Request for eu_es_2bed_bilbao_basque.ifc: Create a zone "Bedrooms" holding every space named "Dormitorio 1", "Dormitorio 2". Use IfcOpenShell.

First a look at what the model holds.

```python
import ifcopenshell

model = ifcopenshell.open("eu_es_2bed_bilbao_basque.ifc")
print(model.schema)
seen = {}
for space in model.by_type("IfcSpace"):
    seen[space.LongName] = seen.get(space.LongName, 0) + 1
for name, count in sorted(seen.items(), key=str):
    print(count, "x", name)
print("zones:", [z.Name for z in model.by_type("IfcZone")][:20])
```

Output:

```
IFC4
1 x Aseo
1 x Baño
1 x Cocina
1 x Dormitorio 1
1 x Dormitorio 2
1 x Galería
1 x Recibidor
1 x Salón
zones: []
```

```python
import ifcopenshell
import ifcopenshell.api.group
import ifcopenshell.api.root

model = ifcopenshell.open("eu_es_2bed_bilbao_basque.ifc")

names = {"Dormitorio 1", "Dormitorio 2"}
spaces = [s for s in model.by_type("IfcSpace") if s.LongName in names]

zone = ifcopenshell.api.root.create_entity(model, ifc_class="IfcZone", name="Bedrooms")
ifcopenshell.api.group.assign_group(model, products=spaces, group=zone)
print(len(spaces), "spaces in", zone.Name)

model.write("eu_es_2bed_bilbao_basque-out.ifc")
```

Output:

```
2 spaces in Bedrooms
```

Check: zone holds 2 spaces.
